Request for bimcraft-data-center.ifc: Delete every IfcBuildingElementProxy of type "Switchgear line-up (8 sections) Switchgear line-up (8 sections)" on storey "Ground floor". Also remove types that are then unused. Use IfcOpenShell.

First a look at what the model holds.

```python
import ifcopenshell
import ifcopenshell.util.element

model = ifcopenshell.open("bimcraft-data-center.ifc")
print(model.schema)
storey = next(s for s in model.by_type("IfcBuildingStorey") if s.Name == "Ground floor")
proxies = [e for e in ifcopenshell.util.element.get_decomposition(storey) if e.is_a("IfcBuildingElementProxy")]
seen = {}
for e in proxies:
    element_type = ifcopenshell.util.element.get_type(e)
    name = element_type.Name if element_type not in (None, e) else None
    seen[name] = seen.get(name, 0) + 1
for name, count in sorted(seen.items(), key=str):
    print(count, "x", name)
```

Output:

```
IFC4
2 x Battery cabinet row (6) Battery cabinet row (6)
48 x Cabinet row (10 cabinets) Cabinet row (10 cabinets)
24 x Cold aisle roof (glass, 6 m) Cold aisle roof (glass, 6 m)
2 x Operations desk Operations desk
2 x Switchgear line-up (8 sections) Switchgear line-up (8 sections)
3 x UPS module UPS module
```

```python
import ifcopenshell
import ifcopenshell.api.root
import ifcopenshell.util.element

model = ifcopenshell.open("bimcraft-data-center.ifc")

storey = next(s for s in model.by_type("IfcBuildingStorey") if s.Name == "Ground floor")
proxies = [e for e in ifcopenshell.util.element.get_decomposition(storey) if e.is_a("IfcBuildingElementProxy")]
targets = [e for e in proxies if (t := ifcopenshell.util.element.get_type(e)) not in (None, e) and t.Name == "Switchgear line-up (8 sections) Switchgear line-up (8 sections)"]
types = {ifcopenshell.util.element.get_type(e) for e in targets} - {None, *targets}

for e in targets:
    ifcopenshell.api.root.remove_product(model, product=e)
print(len(targets), "removed")

unused = [t for t in types if not ifcopenshell.util.element.get_types(t)]
for t in unused:
    ifcopenshell.api.root.remove_product(model, product=t)
print(len(unused), "unused types removed")

model.write("bimcraft-data-center_rev.ifc")
```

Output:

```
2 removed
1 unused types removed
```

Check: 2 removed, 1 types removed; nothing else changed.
